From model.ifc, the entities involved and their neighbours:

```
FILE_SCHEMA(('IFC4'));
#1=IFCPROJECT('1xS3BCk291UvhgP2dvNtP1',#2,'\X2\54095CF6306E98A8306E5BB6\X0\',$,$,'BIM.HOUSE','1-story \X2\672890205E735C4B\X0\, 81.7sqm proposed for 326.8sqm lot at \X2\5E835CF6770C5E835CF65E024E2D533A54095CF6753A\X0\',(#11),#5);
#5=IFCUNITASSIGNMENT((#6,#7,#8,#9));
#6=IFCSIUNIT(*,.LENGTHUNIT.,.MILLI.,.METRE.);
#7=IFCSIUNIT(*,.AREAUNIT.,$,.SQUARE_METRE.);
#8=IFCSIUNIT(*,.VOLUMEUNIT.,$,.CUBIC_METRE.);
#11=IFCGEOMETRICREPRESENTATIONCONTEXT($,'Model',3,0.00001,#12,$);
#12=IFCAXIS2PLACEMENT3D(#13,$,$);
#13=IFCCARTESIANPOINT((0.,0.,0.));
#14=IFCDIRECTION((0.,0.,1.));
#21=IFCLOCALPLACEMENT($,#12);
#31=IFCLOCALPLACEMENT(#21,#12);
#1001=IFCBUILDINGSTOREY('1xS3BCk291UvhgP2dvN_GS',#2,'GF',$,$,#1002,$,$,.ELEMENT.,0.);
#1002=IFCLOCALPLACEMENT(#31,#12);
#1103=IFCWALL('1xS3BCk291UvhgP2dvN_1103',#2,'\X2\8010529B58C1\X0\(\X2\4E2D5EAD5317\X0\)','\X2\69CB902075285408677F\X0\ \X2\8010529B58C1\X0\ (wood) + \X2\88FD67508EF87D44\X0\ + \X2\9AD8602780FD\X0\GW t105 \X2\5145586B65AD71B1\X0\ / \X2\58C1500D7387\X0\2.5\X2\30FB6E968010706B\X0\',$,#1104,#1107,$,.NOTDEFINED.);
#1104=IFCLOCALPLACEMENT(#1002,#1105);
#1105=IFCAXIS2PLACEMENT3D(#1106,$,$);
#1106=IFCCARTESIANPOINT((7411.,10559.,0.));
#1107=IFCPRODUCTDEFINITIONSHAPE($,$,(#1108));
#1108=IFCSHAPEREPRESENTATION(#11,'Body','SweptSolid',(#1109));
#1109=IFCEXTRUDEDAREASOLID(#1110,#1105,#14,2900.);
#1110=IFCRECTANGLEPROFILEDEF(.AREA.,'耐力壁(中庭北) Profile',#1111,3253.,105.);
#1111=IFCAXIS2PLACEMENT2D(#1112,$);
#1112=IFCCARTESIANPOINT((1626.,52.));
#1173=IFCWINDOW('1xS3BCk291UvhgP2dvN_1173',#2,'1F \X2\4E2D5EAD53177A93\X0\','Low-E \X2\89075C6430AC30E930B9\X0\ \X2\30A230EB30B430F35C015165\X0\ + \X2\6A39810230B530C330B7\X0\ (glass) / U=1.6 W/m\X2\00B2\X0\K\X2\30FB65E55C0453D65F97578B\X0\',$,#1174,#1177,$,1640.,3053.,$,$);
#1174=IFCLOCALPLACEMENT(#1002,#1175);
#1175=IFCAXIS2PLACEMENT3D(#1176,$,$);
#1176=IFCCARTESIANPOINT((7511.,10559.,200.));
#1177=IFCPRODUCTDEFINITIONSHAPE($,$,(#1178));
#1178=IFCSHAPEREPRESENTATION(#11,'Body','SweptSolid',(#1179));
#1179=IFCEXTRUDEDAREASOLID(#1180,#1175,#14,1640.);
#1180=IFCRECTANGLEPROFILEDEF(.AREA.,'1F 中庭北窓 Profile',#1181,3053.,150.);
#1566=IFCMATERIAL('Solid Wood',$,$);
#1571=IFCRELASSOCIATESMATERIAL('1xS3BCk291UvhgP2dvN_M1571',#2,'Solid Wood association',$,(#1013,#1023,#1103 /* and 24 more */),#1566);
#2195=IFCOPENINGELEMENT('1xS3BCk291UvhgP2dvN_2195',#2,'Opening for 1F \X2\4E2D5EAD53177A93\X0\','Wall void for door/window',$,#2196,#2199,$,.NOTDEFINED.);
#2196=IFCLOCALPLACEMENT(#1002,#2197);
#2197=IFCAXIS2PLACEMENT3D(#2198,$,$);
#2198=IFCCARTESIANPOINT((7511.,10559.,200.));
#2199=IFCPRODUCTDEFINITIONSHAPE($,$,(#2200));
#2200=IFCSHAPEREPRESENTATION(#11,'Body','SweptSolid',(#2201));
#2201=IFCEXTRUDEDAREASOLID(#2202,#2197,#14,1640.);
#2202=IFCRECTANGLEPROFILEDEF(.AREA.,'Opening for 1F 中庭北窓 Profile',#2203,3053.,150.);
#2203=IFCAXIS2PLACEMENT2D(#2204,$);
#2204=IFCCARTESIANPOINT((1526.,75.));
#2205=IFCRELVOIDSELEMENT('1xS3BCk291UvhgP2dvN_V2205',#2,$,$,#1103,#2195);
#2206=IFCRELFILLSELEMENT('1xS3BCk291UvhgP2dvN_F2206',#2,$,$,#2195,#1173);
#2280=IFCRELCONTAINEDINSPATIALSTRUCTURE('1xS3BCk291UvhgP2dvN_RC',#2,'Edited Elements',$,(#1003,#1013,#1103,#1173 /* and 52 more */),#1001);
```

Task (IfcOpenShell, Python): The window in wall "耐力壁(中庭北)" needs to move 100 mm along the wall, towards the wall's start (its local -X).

```python
import ifcopenshell
import ifcopenshell.api.geometry
import ifcopenshell.util.placement

model = ifcopenshell.open("model.ifc")

window = model.by_guid("1xS3BCk291UvhgP2dvN_1173")
opening = window.FillsVoids[0].RelatingOpeningElement
wall = opening.VoidsElements[0].RelatingBuildingElement

wall_matrix = ifcopenshell.util.placement.get_local_placement(wall.ObjectPlacement)
shift = wall_matrix[:3, 0] * -100.0
before = ifcopenshell.util.placement.get_local_placement(window.ObjectPlacement)[:3, 3].copy()

# The window is not placed relative to its opening, so move both.
for product in (opening, window):
    matrix = ifcopenshell.util.placement.get_local_placement(product.ObjectPlacement)
    matrix[:3, 3] += shift
    ifcopenshell.api.geometry.edit_object_placement(model, product=product, matrix=matrix, is_si=False)

after = ifcopenshell.util.placement.get_local_placement(window.ObjectPlacement)[:3, 3]
print("window moved by", (after - before).round(3) + 0.0)

model.write("model_edited.ifc")
```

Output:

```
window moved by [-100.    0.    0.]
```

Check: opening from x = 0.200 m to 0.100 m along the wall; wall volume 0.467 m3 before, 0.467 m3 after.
